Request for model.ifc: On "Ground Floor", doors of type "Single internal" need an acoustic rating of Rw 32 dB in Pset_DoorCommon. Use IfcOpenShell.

First a look at what the model holds.

```python
import ifcopenshell
import ifcopenshell.util.element

model = ifcopenshell.open("model.ifc")
print(model.schema)
storey = next(s for s in model.by_type("IfcBuildingStorey") if s.Name == "Ground Floor")
doors = [e for e in ifcopenshell.util.element.get_decomposition(storey) if e.is_a("IfcDoor")]
seen = {}
for e in doors:
    element_type = ifcopenshell.util.element.get_type(e)
    key = (element_type.Name if element_type != e and element_type else None, ifcopenshell.util.element.get_pset(e, "Pset_DoorCommon", "AcousticRating"))
    seen[key] = seen.get(key, 0) + 1
for (name, value), count in sorted(seen.items(), key=str):
    print(count, "x", name, "|", value)
```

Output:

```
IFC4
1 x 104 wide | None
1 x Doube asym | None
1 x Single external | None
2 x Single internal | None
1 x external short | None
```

```python
import ifcopenshell
import ifcopenshell.api.pset
import ifcopenshell.util.element

model = ifcopenshell.open("model.ifc")

storey = next(s for s in model.by_type("IfcBuildingStorey") if s.Name == "Ground Floor")
doors = [e for e in ifcopenshell.util.element.get_decomposition(storey) if e.is_a("IfcDoor")]

count = 0
for e in doors:
    element_type = ifcopenshell.util.element.get_type(e)
    if element_type in (None, e) or element_type.Name != "Single internal":
        continue
    # add_pset returns the element's existing set when there is one.
    pset = ifcopenshell.api.pset.add_pset(model, product=e, name="Pset_DoorCommon")
    ifcopenshell.api.pset.edit_pset(model, pset=pset, properties={"AcousticRating": "Rw 32 dB"})
    count += 1

print(count, "doors updated")

model.write("model_v2.ifc")
```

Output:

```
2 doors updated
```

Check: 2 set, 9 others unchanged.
